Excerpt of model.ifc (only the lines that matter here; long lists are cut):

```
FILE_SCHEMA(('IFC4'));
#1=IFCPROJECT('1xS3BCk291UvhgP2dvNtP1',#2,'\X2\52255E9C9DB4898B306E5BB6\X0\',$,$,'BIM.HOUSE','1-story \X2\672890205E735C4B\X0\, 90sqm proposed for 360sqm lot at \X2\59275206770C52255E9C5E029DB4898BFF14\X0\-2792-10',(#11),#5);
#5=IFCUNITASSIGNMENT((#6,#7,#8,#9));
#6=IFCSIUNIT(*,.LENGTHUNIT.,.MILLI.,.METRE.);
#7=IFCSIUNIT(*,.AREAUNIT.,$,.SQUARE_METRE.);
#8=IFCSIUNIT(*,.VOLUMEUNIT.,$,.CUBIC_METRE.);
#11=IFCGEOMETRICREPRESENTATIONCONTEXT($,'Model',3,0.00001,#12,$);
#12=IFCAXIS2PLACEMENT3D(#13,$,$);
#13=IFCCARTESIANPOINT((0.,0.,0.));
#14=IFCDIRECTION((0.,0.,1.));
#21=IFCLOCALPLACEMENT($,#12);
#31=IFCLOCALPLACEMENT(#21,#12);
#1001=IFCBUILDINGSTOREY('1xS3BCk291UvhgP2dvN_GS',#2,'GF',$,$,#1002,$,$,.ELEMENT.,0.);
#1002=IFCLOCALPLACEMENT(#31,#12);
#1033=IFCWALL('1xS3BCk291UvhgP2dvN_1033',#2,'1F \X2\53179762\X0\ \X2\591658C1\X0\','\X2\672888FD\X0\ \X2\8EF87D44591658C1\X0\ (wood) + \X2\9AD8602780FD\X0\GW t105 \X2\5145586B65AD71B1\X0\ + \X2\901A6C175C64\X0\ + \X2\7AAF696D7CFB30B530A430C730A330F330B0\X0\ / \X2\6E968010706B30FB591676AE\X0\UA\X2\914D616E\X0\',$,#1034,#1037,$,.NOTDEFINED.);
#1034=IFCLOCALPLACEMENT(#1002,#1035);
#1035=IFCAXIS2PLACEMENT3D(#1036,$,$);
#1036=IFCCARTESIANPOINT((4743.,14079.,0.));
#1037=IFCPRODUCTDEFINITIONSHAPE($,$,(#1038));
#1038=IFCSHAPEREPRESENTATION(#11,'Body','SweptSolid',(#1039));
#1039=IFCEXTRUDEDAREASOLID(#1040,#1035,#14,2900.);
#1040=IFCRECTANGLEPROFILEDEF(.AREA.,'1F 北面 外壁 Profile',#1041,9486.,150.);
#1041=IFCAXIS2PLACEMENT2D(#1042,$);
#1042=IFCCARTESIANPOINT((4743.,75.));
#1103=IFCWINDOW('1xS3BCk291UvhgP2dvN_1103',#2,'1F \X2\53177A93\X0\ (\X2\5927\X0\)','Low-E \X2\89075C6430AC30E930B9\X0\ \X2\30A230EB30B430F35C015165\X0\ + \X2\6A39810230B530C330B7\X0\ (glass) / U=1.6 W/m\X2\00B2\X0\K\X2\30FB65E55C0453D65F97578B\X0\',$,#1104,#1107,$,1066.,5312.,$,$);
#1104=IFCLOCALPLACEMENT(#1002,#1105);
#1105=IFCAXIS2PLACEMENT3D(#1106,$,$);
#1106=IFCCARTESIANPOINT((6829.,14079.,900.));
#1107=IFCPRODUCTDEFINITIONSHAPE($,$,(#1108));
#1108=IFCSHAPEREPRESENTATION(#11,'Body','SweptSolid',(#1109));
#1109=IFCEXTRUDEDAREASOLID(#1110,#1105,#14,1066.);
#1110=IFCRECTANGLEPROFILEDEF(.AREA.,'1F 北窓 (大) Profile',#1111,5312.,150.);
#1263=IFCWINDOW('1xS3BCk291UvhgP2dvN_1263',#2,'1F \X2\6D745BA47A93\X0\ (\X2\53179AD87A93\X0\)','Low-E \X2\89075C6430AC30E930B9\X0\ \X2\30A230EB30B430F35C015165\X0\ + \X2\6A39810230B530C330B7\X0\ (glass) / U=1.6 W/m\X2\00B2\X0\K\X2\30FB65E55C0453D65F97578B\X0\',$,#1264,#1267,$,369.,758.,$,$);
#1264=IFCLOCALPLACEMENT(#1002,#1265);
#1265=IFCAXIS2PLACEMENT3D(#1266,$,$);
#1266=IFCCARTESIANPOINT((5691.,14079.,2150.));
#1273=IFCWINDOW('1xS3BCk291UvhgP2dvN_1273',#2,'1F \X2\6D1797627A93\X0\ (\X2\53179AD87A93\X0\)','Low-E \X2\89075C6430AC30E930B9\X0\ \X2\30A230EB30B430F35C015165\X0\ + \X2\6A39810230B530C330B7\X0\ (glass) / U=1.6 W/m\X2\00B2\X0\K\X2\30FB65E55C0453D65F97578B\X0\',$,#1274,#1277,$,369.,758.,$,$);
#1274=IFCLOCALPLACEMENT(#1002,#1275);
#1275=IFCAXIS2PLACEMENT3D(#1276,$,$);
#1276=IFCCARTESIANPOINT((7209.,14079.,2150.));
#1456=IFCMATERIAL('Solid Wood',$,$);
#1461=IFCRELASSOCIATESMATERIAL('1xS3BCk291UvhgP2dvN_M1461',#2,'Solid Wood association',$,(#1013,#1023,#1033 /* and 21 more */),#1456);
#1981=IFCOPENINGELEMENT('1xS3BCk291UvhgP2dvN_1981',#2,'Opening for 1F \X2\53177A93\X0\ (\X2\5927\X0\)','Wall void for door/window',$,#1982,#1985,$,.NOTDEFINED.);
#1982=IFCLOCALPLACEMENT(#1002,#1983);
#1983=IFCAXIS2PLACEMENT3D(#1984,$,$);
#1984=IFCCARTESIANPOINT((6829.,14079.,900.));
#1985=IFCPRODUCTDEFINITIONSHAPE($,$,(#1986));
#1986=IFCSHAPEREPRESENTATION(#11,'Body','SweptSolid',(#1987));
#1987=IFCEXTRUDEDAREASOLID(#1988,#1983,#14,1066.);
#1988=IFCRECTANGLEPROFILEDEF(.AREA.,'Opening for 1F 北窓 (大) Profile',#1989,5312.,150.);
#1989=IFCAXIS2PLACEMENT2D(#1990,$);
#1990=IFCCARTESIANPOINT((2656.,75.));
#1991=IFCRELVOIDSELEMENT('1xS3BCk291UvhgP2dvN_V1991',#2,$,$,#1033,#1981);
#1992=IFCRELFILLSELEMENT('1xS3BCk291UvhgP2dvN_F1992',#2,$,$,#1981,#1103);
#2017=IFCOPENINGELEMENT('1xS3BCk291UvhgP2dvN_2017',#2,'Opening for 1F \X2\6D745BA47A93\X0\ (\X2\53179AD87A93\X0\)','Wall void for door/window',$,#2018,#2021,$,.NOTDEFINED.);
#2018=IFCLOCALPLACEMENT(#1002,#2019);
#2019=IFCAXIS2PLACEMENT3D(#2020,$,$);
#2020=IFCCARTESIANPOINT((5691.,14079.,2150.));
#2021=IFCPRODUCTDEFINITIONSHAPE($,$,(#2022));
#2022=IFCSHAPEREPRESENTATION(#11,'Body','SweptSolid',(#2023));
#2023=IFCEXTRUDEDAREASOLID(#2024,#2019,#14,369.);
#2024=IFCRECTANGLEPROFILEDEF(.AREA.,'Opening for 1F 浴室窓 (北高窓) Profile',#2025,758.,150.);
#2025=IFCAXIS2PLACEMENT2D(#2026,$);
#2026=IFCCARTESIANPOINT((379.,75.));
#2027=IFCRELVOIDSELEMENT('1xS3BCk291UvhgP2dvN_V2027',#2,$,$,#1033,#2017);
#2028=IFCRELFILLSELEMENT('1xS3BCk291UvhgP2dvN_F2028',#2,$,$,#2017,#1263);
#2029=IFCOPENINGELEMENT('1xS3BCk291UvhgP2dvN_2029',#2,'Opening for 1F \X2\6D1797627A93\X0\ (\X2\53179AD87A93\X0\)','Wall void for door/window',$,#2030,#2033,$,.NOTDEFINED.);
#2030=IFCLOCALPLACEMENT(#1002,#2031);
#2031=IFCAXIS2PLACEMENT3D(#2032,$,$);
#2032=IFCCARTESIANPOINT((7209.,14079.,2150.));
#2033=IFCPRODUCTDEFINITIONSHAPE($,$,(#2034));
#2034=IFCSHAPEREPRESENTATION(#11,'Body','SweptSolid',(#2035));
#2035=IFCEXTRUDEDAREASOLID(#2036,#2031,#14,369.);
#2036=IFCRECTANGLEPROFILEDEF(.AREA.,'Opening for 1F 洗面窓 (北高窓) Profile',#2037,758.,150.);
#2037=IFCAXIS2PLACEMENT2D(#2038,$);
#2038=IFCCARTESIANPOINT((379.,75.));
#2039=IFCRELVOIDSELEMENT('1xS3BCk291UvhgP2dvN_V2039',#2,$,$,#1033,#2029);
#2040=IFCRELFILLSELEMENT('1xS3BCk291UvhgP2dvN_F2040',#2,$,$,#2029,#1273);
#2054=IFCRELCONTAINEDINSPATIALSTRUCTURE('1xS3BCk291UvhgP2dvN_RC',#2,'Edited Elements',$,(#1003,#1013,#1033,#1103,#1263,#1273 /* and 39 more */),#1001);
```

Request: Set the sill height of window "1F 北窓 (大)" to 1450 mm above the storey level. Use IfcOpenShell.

```python
import numpy as np
import ifcopenshell
import ifcopenshell.api.geometry
import ifcopenshell.geom
import ifcopenshell.util.element
import ifcopenshell.util.placement
import ifcopenshell.util.shape
import ifcopenshell.util.unit

model = ifcopenshell.open("model.ifc")
unit_scale = ifcopenshell.util.unit.calculate_unit_scale(model)

window = model.by_id(1103)
opening = window.FillsVoids[0].RelatingOpeningElement
storey = ifcopenshell.util.element.get_container(window, ifc_class="IfcBuildingStorey")
level = ifcopenshell.util.placement.get_local_placement(storey.ObjectPlacement)[2, 3]

# The opening's origin need not be at the sill, so measure its lowest point.
shape = ifcopenshell.geom.create_shape(ifcopenshell.geom.settings(), opening)
bottom = ifcopenshell.util.shape.get_shape_bottom_elevation(shape, shape.geometry) / unit_scale
dz = level + 1.45 / unit_scale - bottom

shift = np.array([0.0, 0.0, dz])
# The window is not placed relative to its opening, so move both.
for product in (opening, window):
    matrix = ifcopenshell.util.placement.get_local_placement(product.ObjectPlacement)
    matrix[:3, 3] += shift
    ifcopenshell.api.geometry.edit_object_placement(model, product=product, matrix=matrix, is_si=False)

print(f"moved by {dz * unit_scale:+.3f} m")

model.write("model_edited.ifc")
```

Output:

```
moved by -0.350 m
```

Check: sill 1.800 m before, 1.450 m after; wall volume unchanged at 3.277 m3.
